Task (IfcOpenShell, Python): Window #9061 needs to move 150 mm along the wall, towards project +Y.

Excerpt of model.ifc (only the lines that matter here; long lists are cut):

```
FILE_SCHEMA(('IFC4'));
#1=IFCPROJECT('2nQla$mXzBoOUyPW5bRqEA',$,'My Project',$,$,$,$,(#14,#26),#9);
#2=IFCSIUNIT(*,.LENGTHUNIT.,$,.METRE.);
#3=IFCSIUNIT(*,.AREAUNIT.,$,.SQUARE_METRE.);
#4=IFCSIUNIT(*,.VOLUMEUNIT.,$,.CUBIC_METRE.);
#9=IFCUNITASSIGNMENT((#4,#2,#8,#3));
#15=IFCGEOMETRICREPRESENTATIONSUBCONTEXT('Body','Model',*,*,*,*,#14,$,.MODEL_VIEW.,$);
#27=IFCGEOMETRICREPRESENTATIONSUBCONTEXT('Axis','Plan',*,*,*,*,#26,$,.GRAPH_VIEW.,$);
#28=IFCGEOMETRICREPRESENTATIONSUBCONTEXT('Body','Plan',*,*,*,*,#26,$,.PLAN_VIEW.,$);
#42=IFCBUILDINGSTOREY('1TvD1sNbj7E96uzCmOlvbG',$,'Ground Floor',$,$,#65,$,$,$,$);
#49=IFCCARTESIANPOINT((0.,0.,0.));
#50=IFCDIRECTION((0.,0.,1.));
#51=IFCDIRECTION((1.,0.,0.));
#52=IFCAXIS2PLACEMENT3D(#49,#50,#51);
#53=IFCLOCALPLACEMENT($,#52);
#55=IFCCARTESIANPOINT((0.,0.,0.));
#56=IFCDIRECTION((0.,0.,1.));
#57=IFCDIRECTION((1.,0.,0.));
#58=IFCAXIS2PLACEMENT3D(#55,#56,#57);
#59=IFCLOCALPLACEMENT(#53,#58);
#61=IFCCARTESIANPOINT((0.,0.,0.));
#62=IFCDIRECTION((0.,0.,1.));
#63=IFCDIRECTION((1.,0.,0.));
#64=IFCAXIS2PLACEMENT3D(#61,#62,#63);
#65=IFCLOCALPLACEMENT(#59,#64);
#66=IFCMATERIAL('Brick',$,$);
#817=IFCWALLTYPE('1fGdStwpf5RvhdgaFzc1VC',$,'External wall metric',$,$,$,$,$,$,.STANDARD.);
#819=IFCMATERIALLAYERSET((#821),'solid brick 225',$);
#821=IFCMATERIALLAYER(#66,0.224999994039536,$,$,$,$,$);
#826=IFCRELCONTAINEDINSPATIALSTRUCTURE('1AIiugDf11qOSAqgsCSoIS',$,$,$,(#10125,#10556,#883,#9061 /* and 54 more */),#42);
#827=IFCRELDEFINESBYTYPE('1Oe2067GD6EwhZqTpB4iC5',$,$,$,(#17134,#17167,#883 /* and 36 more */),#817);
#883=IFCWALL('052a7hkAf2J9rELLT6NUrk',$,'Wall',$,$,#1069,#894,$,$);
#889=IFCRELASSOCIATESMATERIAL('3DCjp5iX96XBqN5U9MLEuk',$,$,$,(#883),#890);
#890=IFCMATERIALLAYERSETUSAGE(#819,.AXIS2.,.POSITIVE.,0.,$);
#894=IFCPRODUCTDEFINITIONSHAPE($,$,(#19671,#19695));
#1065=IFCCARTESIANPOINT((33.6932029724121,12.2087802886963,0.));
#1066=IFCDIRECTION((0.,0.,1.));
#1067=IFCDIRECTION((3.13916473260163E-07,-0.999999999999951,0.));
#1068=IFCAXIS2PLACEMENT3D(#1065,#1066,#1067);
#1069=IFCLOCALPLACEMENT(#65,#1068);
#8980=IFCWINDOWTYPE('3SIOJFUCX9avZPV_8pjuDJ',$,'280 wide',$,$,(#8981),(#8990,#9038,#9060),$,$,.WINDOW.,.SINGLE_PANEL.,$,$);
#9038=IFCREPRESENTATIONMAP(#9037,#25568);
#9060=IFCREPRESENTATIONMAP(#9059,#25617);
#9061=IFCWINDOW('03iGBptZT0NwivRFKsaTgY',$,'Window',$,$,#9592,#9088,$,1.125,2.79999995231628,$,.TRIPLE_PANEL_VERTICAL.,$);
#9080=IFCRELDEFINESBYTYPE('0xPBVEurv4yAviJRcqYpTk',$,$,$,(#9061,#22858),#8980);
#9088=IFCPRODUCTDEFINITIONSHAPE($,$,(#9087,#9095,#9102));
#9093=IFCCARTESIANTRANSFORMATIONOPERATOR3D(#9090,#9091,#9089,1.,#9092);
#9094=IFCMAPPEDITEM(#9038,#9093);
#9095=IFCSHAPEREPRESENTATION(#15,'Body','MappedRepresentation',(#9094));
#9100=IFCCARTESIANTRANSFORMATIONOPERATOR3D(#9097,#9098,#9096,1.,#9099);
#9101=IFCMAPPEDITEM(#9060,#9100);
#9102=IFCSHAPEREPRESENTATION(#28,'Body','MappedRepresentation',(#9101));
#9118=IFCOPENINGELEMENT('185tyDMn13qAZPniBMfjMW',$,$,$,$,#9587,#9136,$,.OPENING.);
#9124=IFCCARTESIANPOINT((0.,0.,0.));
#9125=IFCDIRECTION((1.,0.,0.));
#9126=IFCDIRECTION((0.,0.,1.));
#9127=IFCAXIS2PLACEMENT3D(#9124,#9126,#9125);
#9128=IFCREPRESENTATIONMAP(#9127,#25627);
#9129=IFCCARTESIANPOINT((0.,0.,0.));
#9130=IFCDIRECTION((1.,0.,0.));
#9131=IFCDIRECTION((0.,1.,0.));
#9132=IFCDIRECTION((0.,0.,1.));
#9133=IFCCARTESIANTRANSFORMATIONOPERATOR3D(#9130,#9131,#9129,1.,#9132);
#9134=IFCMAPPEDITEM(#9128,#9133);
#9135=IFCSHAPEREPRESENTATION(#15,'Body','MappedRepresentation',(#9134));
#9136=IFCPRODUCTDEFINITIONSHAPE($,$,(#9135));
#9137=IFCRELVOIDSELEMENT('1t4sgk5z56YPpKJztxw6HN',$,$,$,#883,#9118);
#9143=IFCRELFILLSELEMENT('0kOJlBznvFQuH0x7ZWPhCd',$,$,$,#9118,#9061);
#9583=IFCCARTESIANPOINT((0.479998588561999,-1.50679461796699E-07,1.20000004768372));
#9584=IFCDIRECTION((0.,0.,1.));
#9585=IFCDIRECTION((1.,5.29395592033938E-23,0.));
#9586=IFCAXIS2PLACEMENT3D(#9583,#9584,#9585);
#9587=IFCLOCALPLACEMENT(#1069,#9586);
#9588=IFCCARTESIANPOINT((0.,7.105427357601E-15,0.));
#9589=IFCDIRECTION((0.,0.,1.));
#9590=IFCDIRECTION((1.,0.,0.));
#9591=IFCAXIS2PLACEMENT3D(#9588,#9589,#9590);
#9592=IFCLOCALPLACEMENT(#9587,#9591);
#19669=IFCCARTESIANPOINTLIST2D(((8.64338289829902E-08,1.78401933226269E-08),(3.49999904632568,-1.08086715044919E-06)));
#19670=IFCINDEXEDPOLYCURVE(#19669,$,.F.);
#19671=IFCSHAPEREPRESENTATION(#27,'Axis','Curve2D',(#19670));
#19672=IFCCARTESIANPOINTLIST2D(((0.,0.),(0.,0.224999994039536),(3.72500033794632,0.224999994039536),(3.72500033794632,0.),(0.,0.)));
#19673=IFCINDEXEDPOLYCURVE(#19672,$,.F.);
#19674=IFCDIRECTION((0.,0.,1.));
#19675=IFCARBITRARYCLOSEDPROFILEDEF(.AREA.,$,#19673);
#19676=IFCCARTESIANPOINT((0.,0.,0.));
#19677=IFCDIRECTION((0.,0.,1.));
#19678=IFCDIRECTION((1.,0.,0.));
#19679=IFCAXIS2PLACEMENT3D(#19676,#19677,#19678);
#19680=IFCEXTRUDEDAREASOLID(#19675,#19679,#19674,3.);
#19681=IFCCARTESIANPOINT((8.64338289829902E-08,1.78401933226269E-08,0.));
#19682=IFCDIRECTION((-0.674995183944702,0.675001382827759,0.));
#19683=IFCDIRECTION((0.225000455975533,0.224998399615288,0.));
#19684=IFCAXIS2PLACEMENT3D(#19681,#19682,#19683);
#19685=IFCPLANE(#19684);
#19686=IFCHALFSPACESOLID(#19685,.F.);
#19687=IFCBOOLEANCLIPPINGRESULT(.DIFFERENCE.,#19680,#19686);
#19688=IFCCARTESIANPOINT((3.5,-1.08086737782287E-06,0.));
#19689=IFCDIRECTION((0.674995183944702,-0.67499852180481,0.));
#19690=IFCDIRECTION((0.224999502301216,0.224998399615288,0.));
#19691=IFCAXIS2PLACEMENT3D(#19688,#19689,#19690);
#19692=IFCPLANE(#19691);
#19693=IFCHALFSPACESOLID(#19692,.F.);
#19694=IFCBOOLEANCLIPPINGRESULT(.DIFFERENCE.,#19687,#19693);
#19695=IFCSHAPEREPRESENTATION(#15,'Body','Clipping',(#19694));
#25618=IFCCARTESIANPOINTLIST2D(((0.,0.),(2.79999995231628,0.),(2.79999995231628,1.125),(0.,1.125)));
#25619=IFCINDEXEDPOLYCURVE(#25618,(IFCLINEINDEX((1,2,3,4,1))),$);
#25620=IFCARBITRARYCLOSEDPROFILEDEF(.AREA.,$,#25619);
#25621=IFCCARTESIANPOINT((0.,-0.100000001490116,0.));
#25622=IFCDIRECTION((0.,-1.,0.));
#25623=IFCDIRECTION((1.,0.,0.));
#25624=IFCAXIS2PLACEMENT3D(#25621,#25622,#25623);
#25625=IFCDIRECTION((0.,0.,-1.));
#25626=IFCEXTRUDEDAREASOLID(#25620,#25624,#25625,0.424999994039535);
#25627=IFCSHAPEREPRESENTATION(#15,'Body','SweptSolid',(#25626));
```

```python
import ifcopenshell
import ifcopenshell.api.geometry
import ifcopenshell.util.placement

model = ifcopenshell.open("model.ifc")

window = model.by_guid("03iGBptZT0NwivRFKsaTgY")
opening = window.FillsVoids[0].RelatingOpeningElement
wall = opening.VoidsElements[0].RelatingBuildingElement

wall_matrix = ifcopenshell.util.placement.get_local_placement(wall.ObjectPlacement)
shift = wall_matrix[:3, 0] * -0.15
before = ifcopenshell.util.placement.get_local_placement(window.ObjectPlacement)[:3, 3].copy()

# The window is placed relative to its opening, so it follows when the opening moves.
matrix = ifcopenshell.util.placement.get_local_placement(opening.ObjectPlacement)
matrix[:3, 3] += shift
ifcopenshell.api.geometry.edit_object_placement(
    model, product=opening, matrix=matrix, is_si=False, should_transform_children=True
)

after = ifcopenshell.util.placement.get_local_placement(window.ObjectPlacement)[:3, 3]
print("window moved by", (after - before).round(3) + 0.0)

model.write("model-out.ifc")
```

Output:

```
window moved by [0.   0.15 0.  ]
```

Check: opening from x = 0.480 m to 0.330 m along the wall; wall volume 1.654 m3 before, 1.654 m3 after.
